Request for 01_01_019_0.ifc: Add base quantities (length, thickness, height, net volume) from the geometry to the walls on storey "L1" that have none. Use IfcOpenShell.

First a look at what the model holds.

```python
import ifcopenshell
import ifcopenshell.util.element
import ifcopenshell.util.unit

model = ifcopenshell.open("01_01_019_0.ifc")
print(model.schema)
for unit_type in ("LENGTHUNIT", "AREAUNIT", "VOLUMEUNIT"):
    print(unit_type, ifcopenshell.util.unit.calculate_unit_scale(model, unit_type))
storey = next(s for s in model.by_type("IfcBuildingStorey") if s.Name == "L1")
walls = [e for e in ifcopenshell.util.element.get_decomposition(storey) if e.is_a("IfcWall")]
for e in sorted(walls, key=lambda e: e.id()):
    print(e.id(), e.is_a(), e.Name, list(ifcopenshell.util.element.get_psets(e, qtos_only=True)), sep=" | ")
```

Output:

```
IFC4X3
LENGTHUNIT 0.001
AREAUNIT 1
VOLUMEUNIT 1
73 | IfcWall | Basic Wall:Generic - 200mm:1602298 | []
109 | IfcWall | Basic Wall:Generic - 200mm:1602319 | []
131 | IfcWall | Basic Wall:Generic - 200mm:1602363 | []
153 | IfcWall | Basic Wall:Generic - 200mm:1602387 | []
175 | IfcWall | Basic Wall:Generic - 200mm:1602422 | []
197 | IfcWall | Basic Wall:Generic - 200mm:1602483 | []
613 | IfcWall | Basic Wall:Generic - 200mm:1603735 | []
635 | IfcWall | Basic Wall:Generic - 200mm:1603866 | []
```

```python
import ifcopenshell
import ifcopenshell.api.pset
import ifcopenshell.geom
import ifcopenshell.util.element
import ifcopenshell.util.shape
import ifcopenshell.util.unit

model = ifcopenshell.open("01_01_019_0.ifc")
unit_scale = ifcopenshell.util.unit.calculate_unit_scale(model)
volume_scale = ifcopenshell.util.unit.calculate_unit_scale(model, "VOLUMEUNIT")
settings = ifcopenshell.geom.settings()

storey = next(s for s in model.by_type("IfcBuildingStorey") if s.Name == "L1")
walls = [e for e in ifcopenshell.util.element.get_decomposition(storey) if e.is_a("IfcWall")]

for e in sorted(walls, key=lambda e: e.id()):
    if ifcopenshell.util.element.get_psets(e, qtos_only=True, should_inherit=False):
        continue
    # Geometry comes back in metres, in the element's own axes.
    shape = ifcopenshell.geom.create_shape(settings, e)
    values = {
        "Length": ifcopenshell.util.shape.get_x(shape.geometry) / unit_scale,
        "Width": ifcopenshell.util.shape.get_y(shape.geometry) / unit_scale,
        "Height": ifcopenshell.util.shape.get_z(shape.geometry) / unit_scale,
        "NetVolume": ifcopenshell.util.shape.get_volume(shape.geometry) / volume_scale,
    }
    qto = ifcopenshell.api.pset.add_qto(model, product=e, name="Qto_WallBaseQuantities")
    ifcopenshell.api.pset.edit_qto(model, qto=qto, properties=values)
    print(e.id(), {k: round(v, 3) for k, v in values.items()})

model.write("01_01_019_0_rev.ifc")
```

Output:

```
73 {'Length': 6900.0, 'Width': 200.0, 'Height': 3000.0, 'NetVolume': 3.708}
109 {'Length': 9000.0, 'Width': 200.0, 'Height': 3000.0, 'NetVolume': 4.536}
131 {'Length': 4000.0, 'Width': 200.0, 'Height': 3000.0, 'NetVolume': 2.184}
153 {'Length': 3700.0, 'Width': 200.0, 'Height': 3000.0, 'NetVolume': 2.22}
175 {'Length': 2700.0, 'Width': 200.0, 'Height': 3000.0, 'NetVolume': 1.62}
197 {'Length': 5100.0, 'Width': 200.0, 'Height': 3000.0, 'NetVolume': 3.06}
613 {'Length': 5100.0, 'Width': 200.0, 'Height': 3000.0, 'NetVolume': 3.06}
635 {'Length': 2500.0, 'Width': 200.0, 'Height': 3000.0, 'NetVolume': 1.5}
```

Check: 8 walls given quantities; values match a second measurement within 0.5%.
